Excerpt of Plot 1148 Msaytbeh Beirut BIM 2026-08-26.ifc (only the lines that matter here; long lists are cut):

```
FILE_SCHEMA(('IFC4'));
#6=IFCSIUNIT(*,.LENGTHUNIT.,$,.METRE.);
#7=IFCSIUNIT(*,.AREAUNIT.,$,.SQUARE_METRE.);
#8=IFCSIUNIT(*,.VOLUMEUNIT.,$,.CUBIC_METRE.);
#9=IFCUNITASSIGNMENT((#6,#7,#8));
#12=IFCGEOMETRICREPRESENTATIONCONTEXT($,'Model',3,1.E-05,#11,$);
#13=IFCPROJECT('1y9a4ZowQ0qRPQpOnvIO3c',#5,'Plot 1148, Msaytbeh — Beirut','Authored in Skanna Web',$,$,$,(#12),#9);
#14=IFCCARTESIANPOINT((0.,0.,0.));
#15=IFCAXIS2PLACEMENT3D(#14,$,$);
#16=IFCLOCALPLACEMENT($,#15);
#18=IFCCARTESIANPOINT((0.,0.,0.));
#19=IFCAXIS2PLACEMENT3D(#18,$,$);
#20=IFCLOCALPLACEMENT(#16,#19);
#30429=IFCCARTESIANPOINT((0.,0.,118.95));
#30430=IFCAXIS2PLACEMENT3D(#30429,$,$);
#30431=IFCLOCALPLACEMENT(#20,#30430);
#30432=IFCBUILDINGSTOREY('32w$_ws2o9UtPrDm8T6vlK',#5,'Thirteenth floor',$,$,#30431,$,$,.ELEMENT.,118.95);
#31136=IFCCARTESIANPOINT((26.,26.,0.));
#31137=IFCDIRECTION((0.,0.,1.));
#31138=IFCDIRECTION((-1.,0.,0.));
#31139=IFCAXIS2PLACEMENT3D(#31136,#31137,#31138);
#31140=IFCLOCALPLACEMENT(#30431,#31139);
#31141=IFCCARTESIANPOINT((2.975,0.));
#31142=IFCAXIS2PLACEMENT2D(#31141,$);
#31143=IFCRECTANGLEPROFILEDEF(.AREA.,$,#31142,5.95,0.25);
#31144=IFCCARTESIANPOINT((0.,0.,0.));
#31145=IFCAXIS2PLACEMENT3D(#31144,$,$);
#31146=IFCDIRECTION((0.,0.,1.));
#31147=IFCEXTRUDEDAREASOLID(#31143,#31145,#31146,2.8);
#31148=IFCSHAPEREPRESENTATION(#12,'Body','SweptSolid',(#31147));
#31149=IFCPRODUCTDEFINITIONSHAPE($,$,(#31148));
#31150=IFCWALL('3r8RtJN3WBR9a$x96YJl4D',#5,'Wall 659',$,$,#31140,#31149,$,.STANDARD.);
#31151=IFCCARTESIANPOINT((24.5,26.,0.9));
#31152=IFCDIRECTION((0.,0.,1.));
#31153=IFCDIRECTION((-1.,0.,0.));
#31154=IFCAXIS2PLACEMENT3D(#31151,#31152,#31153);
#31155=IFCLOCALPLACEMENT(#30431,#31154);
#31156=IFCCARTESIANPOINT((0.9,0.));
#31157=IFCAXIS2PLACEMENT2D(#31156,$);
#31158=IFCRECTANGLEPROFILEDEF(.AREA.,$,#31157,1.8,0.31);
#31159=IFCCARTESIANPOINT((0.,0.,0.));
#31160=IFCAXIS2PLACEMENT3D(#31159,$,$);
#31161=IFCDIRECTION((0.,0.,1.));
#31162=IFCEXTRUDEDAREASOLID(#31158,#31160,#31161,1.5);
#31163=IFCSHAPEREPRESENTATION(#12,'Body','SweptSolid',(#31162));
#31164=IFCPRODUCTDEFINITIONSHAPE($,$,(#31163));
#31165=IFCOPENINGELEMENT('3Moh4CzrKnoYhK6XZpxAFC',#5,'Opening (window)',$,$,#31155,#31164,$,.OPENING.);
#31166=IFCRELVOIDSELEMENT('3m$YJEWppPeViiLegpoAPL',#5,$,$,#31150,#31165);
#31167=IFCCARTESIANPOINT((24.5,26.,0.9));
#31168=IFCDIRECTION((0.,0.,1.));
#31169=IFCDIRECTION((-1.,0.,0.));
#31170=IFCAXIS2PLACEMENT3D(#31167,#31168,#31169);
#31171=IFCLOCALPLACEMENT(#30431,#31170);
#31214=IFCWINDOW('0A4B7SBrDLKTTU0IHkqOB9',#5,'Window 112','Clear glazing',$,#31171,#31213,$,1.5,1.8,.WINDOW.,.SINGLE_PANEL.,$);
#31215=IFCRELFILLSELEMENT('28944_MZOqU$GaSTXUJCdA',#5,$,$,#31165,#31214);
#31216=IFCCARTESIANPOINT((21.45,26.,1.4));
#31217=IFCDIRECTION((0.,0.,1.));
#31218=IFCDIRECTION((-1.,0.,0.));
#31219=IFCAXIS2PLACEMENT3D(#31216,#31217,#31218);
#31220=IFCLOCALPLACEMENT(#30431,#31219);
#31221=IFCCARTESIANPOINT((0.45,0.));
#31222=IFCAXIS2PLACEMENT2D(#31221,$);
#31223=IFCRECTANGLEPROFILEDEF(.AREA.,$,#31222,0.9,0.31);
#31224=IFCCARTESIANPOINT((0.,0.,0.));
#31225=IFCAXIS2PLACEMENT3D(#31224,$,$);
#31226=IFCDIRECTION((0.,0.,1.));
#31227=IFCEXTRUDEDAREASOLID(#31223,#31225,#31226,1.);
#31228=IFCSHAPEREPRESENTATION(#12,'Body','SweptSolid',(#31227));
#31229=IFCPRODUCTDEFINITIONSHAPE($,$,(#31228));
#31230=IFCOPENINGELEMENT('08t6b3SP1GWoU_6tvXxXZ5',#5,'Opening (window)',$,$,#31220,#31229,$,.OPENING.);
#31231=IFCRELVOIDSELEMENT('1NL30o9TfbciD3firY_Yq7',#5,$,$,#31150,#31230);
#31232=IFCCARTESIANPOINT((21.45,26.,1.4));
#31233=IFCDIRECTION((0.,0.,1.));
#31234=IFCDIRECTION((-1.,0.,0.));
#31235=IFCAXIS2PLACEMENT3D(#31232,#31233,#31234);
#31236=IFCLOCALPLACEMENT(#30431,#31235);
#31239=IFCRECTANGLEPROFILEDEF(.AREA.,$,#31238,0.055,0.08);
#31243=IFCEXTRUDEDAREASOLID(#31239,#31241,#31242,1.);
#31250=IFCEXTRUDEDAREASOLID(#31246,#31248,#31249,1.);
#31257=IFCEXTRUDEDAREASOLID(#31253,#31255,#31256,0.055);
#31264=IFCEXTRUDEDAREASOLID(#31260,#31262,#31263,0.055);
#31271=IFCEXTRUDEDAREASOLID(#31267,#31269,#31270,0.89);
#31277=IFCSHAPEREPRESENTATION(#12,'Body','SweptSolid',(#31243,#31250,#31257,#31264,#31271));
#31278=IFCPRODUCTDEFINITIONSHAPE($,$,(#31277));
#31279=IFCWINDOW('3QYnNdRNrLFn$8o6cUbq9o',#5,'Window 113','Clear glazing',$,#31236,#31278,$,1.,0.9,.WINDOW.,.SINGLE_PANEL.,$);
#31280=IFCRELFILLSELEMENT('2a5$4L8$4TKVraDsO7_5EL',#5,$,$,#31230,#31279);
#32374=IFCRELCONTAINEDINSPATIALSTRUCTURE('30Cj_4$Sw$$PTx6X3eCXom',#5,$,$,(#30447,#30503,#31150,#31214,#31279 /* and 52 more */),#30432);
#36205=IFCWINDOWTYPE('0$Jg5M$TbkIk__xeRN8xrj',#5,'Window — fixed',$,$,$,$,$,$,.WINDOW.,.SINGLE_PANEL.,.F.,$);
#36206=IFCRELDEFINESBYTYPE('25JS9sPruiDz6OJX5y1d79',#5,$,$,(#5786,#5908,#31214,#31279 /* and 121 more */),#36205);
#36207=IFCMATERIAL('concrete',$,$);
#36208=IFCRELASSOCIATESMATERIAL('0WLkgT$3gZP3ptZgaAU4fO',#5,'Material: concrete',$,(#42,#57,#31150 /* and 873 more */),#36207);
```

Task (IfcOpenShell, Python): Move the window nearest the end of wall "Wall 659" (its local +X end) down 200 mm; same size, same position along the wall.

```python
import numpy as np
import ifcopenshell
import ifcopenshell.api.geometry
import ifcopenshell.util.placement
import ifcopenshell.util.unit

model = ifcopenshell.open("Plot 1148 Msaytbeh Beirut BIM 2026-08-26.ifc")
unit_scale = ifcopenshell.util.unit.calculate_unit_scale(model)

window = model.by_guid("3QYnNdRNrLFn$8o6cUbq9o")
opening = window.FillsVoids[0].RelatingOpeningElement
dz = -0.2 / unit_scale

shift = np.array([0.0, 0.0, dz])
# The window is not placed relative to its opening, so move both.
for product in (opening, window):
    matrix = ifcopenshell.util.placement.get_local_placement(product.ObjectPlacement)
    matrix[:3, 3] += shift
    ifcopenshell.api.geometry.edit_object_placement(model, product=product, matrix=matrix, is_si=False)

print(f"moved by {dz * unit_scale:+.3f} m")

model.write("Plot 1148 Msaytbeh Beirut BIM 2026-08-26-out.ifc")
```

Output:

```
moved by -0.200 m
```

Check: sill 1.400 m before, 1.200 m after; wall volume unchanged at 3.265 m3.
